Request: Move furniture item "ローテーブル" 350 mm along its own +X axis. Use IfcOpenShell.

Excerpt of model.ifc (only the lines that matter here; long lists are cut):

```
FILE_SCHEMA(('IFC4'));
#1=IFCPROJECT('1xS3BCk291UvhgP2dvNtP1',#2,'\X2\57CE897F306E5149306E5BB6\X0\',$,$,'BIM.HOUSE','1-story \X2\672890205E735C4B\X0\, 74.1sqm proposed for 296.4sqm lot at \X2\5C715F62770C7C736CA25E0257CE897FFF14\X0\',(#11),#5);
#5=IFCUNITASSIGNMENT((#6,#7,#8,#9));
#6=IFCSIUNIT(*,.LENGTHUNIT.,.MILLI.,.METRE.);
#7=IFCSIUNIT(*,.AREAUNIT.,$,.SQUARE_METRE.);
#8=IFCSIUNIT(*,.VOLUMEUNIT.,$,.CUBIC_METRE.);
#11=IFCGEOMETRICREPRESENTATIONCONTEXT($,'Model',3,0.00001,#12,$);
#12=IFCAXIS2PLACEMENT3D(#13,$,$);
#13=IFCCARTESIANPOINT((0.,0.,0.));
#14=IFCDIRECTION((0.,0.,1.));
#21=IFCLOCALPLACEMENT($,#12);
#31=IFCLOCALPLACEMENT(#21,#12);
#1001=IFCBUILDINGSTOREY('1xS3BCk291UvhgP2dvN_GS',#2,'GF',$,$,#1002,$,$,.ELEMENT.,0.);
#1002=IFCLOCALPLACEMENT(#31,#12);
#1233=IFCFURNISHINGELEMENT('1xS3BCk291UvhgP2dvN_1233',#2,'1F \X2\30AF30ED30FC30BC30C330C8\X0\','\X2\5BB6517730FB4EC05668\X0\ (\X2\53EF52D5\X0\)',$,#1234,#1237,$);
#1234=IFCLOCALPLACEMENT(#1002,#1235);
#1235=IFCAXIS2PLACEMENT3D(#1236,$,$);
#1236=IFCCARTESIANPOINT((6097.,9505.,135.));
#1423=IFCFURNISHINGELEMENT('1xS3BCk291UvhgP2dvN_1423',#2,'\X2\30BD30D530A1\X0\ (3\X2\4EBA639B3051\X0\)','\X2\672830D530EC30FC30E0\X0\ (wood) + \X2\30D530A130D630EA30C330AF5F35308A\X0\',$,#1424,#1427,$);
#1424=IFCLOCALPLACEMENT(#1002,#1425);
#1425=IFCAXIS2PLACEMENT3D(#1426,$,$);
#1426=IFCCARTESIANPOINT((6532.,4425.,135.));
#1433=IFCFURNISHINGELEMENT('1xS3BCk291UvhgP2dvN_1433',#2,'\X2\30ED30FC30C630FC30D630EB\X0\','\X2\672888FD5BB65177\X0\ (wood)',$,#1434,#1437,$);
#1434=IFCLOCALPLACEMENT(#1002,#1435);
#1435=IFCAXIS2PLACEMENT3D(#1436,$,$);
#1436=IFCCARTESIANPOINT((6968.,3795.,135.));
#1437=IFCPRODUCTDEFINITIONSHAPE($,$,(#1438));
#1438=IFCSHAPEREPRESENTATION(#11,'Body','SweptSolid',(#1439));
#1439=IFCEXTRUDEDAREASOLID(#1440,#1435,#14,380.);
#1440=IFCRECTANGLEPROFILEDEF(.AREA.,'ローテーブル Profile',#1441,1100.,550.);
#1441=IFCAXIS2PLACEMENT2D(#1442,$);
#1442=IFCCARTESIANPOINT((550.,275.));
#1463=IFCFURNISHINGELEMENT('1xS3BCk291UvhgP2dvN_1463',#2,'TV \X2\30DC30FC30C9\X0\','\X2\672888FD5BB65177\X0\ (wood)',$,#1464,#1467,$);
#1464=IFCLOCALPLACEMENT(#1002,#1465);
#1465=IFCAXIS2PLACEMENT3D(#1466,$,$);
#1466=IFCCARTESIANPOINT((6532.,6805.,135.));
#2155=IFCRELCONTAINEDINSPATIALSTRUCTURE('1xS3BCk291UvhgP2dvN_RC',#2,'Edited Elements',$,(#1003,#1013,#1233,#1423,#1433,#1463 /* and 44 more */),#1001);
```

```python
import ifcopenshell
import ifcopenshell.api.geometry
import ifcopenshell.util.placement

model = ifcopenshell.open("model.ifc")

item = model.by_guid("1xS3BCk291UvhgP2dvN_1433")
matrix = ifcopenshell.util.placement.get_local_placement(item.ObjectPlacement)
matrix[:3, 3] += matrix[:3, 0] * 350.0
ifcopenshell.api.geometry.edit_object_placement(model, product=item, matrix=matrix, is_si=False)

print(ifcopenshell.util.placement.get_local_placement(item.ObjectPlacement).round(3) + 0.0)

model.write("model_updated.ifc")
```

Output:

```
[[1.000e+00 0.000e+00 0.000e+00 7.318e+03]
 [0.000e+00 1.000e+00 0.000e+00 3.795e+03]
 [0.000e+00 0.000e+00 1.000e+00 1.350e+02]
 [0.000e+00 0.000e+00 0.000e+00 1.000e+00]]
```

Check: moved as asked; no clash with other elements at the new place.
